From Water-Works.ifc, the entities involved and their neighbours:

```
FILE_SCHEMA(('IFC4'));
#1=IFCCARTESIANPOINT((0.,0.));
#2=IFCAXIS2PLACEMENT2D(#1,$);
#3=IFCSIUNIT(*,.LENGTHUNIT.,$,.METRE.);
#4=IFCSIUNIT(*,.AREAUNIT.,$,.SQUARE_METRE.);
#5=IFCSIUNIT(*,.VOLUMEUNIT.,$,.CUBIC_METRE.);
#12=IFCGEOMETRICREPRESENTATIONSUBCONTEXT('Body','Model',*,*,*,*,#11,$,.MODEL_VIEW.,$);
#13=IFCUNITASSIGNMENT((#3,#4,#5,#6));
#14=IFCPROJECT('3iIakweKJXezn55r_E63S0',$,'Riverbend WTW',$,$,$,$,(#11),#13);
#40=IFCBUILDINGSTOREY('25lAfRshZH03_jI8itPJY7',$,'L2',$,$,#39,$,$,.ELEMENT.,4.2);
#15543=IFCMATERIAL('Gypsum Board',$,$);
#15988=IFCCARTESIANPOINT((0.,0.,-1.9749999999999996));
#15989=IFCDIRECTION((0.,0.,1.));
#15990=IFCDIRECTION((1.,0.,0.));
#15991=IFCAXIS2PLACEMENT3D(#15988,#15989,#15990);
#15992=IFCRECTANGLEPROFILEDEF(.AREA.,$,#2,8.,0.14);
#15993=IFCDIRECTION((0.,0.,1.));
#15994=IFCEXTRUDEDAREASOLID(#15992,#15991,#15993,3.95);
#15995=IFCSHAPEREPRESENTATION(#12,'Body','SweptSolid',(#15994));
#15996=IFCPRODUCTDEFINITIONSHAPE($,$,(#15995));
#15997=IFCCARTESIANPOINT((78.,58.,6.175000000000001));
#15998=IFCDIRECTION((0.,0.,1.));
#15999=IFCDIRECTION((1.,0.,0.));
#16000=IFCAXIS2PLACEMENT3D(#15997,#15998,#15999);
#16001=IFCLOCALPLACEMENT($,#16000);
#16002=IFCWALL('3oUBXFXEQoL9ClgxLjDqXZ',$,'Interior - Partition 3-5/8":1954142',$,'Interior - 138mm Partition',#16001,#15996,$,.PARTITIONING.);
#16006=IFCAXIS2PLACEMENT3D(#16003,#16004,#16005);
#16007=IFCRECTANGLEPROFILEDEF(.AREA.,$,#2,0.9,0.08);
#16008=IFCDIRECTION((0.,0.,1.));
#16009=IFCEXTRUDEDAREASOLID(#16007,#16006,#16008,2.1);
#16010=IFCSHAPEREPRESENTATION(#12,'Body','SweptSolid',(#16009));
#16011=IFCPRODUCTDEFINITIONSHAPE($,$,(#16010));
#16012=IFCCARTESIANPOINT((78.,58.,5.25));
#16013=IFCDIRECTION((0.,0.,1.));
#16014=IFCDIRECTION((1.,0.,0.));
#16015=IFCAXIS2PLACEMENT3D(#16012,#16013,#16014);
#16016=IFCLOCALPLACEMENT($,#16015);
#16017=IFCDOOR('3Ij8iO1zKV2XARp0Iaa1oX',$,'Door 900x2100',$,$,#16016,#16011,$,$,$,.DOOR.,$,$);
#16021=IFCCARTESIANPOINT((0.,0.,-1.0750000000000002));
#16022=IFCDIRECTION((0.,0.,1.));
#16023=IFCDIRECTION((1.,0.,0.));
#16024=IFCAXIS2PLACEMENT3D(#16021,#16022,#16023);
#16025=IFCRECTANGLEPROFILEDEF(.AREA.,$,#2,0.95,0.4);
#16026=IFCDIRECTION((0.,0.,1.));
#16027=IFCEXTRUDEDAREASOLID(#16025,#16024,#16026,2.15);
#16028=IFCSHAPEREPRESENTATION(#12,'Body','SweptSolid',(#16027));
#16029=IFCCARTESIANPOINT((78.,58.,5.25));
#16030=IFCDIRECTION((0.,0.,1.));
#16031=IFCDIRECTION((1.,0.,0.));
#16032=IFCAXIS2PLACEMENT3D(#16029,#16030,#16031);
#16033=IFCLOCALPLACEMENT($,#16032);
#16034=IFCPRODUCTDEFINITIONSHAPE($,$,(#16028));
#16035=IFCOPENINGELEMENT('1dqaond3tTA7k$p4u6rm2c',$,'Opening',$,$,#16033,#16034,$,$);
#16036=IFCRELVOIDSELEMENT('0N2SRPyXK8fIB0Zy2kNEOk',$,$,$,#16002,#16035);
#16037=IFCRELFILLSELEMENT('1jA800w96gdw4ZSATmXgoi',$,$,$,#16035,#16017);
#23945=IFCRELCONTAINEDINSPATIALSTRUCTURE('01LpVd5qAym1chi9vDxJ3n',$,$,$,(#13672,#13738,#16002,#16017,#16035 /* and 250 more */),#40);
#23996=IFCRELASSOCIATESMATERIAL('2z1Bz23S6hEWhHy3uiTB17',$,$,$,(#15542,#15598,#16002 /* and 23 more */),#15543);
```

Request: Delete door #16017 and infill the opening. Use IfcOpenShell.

```python
import ifcopenshell
import ifcopenshell.api.feature
import ifcopenshell.api.root
import ifcopenshell.geom
import ifcopenshell.util.shape

model = ifcopenshell.open("Water-Works.ifc")
settings = ifcopenshell.geom.settings()


def volume(element):
    """Net volume in cubic metres, openings subtracted."""
    shape = ifcopenshell.geom.create_shape(settings, element)
    return ifcopenshell.util.shape.get_volume(shape.geometry)


door = model.by_guid("3Ij8iO1zKV2XARp0Iaa1oX")
opening = door.FillsVoids[0].RelatingOpeningElement
wall = opening.VoidsElements[0].RelatingBuildingElement
before = volume(wall)

ifcopenshell.api.root.remove_product(model, product=door)
ifcopenshell.api.feature.remove_feature(model, feature=opening)

after = volume(wall)

print(f"wall volume {before:.3f} -> {after:.3f} m3")

model.write("Water-Works_rev.ifc")
```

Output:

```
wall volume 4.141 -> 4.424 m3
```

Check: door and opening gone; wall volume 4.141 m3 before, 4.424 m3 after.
